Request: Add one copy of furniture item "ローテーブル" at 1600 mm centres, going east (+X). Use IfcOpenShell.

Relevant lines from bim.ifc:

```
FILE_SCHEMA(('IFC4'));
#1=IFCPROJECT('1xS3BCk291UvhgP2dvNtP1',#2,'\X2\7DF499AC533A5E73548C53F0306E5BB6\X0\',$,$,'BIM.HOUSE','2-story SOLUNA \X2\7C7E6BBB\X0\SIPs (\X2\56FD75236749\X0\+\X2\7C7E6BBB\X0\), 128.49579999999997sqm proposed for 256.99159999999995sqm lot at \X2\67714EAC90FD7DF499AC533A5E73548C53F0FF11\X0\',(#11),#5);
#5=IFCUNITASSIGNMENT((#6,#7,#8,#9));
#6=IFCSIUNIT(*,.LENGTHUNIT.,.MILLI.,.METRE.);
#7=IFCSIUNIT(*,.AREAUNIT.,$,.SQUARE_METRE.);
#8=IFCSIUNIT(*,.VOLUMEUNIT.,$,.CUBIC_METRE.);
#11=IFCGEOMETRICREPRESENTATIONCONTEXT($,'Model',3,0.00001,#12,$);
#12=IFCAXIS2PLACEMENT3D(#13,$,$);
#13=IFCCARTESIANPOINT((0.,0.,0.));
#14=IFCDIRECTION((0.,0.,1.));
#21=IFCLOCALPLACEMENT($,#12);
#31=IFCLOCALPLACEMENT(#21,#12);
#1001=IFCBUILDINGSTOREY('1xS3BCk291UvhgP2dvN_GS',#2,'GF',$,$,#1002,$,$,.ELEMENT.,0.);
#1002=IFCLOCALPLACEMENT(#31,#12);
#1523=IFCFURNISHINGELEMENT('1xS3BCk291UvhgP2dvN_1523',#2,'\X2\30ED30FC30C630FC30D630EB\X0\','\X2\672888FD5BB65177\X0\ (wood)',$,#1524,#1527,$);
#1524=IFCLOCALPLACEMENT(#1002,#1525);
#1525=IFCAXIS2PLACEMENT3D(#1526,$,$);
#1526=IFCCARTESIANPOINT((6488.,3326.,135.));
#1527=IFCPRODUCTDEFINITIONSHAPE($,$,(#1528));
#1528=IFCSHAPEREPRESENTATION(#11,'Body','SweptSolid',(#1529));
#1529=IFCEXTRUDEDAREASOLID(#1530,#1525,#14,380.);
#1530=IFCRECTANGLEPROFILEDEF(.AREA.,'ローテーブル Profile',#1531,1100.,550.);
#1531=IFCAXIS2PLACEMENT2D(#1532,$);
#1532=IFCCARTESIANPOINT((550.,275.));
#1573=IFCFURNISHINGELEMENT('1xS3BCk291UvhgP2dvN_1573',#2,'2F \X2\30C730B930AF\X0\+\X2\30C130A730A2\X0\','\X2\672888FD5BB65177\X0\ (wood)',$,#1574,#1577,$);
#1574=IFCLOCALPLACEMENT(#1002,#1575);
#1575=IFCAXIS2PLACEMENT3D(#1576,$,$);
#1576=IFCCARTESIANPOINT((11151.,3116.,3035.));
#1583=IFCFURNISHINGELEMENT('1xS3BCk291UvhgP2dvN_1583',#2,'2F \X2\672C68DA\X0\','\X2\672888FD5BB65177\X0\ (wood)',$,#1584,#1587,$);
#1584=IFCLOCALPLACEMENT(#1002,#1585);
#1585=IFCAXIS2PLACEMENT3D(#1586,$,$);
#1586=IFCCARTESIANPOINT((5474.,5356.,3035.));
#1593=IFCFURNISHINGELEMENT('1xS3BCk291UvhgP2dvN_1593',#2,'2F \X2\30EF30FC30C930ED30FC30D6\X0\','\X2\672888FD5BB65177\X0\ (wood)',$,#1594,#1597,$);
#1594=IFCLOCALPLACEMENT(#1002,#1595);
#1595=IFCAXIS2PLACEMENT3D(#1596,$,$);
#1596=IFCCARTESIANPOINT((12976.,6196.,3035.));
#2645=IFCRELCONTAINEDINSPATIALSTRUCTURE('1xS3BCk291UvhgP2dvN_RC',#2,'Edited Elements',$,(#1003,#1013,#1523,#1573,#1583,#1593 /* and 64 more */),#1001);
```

```python
import numpy as np
import ifcopenshell
import ifcopenshell.api.geometry
import ifcopenshell.api.root
import ifcopenshell.util.element
import ifcopenshell.util.placement

model = ifcopenshell.open("bim.ifc")


def reuse_history(source, copy):
    """copy_class also copies each property set's owner history, people and application; keep the originals."""
    for rel in copy.IsDefinedBy:
        if rel.is_a("IfcRelDefinesByProperties") and (history := rel.RelatingPropertyDefinition.OwnerHistory):
            rel.RelatingPropertyDefinition.OwnerHistory = source.OwnerHistory
            ifcopenshell.util.element.remove_deep2(model, history)


source = model.by_guid("1xS3BCk291UvhgP2dvN_1523")
base = ifcopenshell.util.placement.get_local_placement(source.ObjectPlacement)
step = np.array([1.0, 0.0, 0.0]) * 1600.0

for i in range(1, 2):
    copy = ifcopenshell.api.root.copy_class(model, product=source)
    copy.Representation = ifcopenshell.util.element.copy_deep(
        model, source.Representation, exclude=["IfcGeometricRepresentationContext", "IfcRepresentationMap"]
    )
    reuse_history(source, copy)
    matrix = base.copy()
    matrix[:3, 3] += i * step
    print("added at", matrix[:3, 3].round(3) + 0.0)
    ifcopenshell.api.geometry.edit_object_placement(model, product=copy, matrix=matrix, is_si=False)

model.write("bim_v2.ifc")
```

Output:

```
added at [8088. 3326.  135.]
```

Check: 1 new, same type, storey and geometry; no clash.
